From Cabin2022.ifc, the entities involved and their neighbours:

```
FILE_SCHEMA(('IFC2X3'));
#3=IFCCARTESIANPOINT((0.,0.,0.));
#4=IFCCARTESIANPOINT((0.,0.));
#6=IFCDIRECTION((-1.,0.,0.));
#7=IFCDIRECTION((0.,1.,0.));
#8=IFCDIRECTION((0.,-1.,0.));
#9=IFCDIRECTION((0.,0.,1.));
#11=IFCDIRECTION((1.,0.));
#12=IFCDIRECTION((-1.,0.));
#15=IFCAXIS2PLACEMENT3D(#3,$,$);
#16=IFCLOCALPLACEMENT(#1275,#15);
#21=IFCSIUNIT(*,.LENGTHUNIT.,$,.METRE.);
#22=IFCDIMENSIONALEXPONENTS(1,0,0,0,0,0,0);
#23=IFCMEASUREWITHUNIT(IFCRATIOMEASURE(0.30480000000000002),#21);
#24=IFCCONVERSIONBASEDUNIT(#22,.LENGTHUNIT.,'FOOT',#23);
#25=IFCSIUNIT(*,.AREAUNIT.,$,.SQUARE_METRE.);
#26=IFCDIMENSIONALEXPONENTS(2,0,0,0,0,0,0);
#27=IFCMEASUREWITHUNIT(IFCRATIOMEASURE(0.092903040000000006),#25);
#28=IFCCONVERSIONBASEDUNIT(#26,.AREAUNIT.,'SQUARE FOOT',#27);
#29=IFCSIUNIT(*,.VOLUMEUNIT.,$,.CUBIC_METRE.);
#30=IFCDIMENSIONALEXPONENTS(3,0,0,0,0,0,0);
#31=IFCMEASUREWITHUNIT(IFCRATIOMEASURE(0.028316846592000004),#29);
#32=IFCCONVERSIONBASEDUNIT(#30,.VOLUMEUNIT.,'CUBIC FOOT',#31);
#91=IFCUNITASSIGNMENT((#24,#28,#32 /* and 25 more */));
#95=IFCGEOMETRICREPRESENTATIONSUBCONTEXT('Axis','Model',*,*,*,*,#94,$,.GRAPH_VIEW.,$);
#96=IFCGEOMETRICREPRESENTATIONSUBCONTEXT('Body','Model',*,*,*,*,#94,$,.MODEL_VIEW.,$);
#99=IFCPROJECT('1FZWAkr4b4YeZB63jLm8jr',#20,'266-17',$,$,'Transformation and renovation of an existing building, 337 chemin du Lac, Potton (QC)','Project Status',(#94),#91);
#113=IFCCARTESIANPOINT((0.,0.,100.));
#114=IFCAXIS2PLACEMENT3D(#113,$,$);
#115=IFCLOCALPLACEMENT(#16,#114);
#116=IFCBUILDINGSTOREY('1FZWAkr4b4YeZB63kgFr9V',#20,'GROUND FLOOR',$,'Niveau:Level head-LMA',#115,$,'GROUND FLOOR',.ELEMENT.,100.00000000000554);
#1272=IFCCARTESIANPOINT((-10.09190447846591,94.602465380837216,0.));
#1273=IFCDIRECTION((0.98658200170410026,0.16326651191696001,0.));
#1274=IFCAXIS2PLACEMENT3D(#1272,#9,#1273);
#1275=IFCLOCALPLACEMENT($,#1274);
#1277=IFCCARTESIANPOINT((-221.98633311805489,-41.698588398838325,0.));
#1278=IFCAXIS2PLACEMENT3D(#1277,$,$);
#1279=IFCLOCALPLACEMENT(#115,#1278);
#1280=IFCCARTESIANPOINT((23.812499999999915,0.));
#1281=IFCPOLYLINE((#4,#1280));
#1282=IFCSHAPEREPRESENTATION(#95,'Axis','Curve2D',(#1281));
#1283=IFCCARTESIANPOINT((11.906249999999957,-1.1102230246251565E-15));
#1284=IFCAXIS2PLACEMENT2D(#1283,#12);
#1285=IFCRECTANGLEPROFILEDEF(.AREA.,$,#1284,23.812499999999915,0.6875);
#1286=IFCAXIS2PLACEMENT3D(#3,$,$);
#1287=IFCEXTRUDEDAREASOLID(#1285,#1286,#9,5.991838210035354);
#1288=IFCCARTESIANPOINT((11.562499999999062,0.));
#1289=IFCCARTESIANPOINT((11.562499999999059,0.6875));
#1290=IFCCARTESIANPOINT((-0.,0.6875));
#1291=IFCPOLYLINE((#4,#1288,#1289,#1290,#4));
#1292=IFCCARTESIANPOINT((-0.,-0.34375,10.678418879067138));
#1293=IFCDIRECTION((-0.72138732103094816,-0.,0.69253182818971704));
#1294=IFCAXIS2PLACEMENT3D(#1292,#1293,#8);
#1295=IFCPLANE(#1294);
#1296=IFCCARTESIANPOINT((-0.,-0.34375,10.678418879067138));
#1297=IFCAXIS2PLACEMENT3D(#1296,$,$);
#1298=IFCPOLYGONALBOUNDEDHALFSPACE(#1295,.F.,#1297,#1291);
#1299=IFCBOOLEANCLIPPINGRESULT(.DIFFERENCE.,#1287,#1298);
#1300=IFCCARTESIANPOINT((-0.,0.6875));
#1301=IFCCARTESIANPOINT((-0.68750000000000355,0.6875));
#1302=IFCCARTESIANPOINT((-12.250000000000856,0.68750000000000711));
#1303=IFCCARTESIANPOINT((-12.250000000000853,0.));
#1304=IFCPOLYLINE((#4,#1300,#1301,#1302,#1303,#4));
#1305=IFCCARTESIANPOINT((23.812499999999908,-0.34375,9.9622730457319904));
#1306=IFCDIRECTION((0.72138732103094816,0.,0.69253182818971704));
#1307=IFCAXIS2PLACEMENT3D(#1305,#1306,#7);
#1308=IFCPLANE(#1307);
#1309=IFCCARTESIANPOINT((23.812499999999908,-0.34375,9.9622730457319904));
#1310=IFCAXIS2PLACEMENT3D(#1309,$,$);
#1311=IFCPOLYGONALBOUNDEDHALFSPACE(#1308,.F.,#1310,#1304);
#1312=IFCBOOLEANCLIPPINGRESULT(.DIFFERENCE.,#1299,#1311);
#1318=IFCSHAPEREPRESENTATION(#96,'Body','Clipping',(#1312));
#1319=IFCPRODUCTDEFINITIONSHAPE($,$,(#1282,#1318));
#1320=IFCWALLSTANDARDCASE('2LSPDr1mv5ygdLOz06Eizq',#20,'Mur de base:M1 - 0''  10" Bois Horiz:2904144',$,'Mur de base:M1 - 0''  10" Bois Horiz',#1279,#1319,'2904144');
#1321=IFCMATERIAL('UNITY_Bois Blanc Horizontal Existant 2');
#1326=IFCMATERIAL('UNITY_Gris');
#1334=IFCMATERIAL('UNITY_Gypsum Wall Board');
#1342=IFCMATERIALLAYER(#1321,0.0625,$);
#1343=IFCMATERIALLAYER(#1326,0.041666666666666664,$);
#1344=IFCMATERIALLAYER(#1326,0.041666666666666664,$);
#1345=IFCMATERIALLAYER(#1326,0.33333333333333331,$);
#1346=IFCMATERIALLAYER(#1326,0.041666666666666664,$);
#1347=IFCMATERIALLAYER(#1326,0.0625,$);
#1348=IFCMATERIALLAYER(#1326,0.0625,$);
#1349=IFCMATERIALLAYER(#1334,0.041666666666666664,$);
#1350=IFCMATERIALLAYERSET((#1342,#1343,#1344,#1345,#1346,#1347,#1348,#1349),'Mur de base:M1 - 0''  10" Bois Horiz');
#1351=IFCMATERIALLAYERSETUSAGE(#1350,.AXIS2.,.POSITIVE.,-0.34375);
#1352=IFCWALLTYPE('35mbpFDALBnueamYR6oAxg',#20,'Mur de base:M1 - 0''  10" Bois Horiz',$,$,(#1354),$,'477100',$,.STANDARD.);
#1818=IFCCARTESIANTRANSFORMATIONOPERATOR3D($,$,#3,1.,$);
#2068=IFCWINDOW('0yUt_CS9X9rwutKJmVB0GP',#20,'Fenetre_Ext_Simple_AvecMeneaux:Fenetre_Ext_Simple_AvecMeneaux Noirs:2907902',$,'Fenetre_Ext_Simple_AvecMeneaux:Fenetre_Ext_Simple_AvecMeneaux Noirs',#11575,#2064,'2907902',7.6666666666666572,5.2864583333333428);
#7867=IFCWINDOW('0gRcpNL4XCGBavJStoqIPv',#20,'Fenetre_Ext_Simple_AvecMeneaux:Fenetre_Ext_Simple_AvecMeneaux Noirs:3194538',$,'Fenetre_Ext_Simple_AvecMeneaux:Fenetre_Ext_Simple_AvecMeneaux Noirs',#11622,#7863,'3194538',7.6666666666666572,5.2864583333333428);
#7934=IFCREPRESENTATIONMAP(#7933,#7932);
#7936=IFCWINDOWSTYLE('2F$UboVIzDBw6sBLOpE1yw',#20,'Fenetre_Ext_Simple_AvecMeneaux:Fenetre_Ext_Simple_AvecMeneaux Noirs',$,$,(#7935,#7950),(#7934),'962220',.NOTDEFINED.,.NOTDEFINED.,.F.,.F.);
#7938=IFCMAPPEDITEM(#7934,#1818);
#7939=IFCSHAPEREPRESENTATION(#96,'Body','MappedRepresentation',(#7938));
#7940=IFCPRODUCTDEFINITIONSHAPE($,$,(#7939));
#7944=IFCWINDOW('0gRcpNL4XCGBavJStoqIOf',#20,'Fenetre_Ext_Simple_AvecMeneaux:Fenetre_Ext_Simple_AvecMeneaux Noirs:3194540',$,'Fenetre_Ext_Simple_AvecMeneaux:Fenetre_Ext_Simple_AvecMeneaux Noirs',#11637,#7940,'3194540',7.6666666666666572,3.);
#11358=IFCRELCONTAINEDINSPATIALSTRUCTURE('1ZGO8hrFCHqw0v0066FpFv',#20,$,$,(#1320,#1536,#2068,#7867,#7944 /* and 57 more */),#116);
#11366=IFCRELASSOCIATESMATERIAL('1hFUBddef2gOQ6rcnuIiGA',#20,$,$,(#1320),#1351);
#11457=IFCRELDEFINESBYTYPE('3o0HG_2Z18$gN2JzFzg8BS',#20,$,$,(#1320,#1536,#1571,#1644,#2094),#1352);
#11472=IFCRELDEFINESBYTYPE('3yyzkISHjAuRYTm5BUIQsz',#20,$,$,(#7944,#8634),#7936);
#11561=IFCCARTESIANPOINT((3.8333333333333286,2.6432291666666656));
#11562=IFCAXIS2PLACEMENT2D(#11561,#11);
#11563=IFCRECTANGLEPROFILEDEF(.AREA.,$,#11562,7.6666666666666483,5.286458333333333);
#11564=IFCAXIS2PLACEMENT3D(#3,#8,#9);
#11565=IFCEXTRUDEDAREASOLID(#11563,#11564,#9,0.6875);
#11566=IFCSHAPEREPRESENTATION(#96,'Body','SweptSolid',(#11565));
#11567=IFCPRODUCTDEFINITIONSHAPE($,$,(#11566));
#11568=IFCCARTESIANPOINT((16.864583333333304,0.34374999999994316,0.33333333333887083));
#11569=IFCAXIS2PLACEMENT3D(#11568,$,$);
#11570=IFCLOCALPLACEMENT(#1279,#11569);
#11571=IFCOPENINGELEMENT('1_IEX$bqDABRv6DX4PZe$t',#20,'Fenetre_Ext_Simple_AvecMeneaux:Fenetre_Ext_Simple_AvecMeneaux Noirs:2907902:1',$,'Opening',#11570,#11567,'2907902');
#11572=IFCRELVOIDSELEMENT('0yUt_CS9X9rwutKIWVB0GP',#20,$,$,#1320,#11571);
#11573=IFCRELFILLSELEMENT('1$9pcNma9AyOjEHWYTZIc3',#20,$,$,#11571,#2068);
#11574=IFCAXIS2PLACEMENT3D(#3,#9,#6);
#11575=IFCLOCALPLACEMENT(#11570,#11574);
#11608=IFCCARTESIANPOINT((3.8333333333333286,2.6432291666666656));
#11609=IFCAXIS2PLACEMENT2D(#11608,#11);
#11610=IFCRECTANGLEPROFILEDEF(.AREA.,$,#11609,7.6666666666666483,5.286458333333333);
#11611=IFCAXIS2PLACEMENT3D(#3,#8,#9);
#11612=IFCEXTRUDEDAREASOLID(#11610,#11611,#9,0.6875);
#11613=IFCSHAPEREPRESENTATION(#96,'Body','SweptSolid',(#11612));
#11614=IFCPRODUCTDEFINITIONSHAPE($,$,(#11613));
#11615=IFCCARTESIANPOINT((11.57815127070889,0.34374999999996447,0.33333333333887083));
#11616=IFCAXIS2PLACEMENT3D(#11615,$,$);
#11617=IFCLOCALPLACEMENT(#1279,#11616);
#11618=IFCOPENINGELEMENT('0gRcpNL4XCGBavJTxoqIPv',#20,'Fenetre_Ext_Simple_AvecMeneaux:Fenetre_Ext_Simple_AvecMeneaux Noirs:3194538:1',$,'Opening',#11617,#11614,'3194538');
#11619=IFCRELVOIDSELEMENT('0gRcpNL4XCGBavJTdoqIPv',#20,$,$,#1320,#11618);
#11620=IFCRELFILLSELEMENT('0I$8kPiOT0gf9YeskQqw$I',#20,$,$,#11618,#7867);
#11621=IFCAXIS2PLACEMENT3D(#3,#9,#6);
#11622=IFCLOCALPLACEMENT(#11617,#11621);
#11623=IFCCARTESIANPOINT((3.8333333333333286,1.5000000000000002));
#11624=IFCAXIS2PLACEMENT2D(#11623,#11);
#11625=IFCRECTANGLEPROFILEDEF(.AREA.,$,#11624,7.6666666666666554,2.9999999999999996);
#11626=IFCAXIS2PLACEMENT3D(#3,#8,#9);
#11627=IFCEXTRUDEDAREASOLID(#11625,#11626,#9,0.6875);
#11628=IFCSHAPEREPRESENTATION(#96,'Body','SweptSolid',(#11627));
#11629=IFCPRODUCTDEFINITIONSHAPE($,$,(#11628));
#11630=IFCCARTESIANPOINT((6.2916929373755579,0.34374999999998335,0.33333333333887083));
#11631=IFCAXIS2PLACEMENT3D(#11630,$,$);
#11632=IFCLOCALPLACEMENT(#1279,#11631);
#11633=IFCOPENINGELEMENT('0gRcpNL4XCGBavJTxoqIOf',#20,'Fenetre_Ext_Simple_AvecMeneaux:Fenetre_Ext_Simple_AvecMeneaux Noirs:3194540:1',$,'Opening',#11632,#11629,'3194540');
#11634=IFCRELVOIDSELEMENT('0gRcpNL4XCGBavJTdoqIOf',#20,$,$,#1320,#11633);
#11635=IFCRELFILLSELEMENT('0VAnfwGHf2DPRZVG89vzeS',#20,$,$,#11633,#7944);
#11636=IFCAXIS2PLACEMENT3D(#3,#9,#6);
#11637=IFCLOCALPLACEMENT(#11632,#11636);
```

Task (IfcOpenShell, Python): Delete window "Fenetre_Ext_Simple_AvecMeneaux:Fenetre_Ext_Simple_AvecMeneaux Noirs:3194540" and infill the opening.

```python
import ifcopenshell
import ifcopenshell.api.feature
import ifcopenshell.api.root
import ifcopenshell.geom
import ifcopenshell.util.shape

model = ifcopenshell.open("Cabin2022.ifc")
settings = ifcopenshell.geom.settings()


def volume(element):
    """Net volume in cubic metres, openings subtracted."""
    shape = ifcopenshell.geom.create_shape(settings, element)
    return ifcopenshell.util.shape.get_volume(shape.geometry)


window = model.by_guid("0gRcpNL4XCGBavJStoqIOf")
opening = window.FillsVoids[0].RelatingOpeningElement
wall = opening.VoidsElements[0].RelatingBuildingElement
before = volume(wall)

ifcopenshell.api.root.remove_product(model, product=window)
ifcopenshell.api.feature.remove_feature(model, feature=opening)

after = volume(wall)

print(f"wall volume {before:.3f} -> {after:.3f} m3")

model.write("Cabin2022_updated.ifc")
```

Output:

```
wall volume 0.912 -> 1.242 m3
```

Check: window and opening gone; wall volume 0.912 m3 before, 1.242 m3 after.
